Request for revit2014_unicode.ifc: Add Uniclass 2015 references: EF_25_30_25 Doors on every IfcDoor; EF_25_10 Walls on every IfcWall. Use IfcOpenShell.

First a look at what the model holds.

```python
import ifcopenshell

model = ifcopenshell.open("revit2014_unicode.ifc")
print(model.schema)
print("classifications:", [c.Name for c in model.by_type("IfcClassification")])
for ifc_class in ("IfcDoor", "IfcRoof", "IfcStair", "IfcWall", "IfcWindow"):
    print(ifc_class, len(model.by_type(ifc_class)))
```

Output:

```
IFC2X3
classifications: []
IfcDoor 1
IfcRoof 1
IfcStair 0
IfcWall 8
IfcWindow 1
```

```python
import ifcopenshell
import ifcopenshell.api.classification

model = ifcopenshell.open("revit2014_unicode.ifc")

# IFC2X3 requires Source and Edition and has no link from the project to the system.
system = model.create_entity("IfcClassification", Source="NBS", Edition="2015", Name="Uniclass 2015")

codes = {
    "IfcDoor": ("EF_25_30_25", "Doors"),
    "IfcWall": ("EF_25_10", "Walls"),
}
for ifc_class, (code, name) in codes.items():
    products = model.by_type(ifc_class)
    ifcopenshell.api.classification.add_reference(
        model, products=products, classification=system, identification=code, name=name
    )
    print(code, len(products))

model.write("revit2014_unicode-out.ifc")
```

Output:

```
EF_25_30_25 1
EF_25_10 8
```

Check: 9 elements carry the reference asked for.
